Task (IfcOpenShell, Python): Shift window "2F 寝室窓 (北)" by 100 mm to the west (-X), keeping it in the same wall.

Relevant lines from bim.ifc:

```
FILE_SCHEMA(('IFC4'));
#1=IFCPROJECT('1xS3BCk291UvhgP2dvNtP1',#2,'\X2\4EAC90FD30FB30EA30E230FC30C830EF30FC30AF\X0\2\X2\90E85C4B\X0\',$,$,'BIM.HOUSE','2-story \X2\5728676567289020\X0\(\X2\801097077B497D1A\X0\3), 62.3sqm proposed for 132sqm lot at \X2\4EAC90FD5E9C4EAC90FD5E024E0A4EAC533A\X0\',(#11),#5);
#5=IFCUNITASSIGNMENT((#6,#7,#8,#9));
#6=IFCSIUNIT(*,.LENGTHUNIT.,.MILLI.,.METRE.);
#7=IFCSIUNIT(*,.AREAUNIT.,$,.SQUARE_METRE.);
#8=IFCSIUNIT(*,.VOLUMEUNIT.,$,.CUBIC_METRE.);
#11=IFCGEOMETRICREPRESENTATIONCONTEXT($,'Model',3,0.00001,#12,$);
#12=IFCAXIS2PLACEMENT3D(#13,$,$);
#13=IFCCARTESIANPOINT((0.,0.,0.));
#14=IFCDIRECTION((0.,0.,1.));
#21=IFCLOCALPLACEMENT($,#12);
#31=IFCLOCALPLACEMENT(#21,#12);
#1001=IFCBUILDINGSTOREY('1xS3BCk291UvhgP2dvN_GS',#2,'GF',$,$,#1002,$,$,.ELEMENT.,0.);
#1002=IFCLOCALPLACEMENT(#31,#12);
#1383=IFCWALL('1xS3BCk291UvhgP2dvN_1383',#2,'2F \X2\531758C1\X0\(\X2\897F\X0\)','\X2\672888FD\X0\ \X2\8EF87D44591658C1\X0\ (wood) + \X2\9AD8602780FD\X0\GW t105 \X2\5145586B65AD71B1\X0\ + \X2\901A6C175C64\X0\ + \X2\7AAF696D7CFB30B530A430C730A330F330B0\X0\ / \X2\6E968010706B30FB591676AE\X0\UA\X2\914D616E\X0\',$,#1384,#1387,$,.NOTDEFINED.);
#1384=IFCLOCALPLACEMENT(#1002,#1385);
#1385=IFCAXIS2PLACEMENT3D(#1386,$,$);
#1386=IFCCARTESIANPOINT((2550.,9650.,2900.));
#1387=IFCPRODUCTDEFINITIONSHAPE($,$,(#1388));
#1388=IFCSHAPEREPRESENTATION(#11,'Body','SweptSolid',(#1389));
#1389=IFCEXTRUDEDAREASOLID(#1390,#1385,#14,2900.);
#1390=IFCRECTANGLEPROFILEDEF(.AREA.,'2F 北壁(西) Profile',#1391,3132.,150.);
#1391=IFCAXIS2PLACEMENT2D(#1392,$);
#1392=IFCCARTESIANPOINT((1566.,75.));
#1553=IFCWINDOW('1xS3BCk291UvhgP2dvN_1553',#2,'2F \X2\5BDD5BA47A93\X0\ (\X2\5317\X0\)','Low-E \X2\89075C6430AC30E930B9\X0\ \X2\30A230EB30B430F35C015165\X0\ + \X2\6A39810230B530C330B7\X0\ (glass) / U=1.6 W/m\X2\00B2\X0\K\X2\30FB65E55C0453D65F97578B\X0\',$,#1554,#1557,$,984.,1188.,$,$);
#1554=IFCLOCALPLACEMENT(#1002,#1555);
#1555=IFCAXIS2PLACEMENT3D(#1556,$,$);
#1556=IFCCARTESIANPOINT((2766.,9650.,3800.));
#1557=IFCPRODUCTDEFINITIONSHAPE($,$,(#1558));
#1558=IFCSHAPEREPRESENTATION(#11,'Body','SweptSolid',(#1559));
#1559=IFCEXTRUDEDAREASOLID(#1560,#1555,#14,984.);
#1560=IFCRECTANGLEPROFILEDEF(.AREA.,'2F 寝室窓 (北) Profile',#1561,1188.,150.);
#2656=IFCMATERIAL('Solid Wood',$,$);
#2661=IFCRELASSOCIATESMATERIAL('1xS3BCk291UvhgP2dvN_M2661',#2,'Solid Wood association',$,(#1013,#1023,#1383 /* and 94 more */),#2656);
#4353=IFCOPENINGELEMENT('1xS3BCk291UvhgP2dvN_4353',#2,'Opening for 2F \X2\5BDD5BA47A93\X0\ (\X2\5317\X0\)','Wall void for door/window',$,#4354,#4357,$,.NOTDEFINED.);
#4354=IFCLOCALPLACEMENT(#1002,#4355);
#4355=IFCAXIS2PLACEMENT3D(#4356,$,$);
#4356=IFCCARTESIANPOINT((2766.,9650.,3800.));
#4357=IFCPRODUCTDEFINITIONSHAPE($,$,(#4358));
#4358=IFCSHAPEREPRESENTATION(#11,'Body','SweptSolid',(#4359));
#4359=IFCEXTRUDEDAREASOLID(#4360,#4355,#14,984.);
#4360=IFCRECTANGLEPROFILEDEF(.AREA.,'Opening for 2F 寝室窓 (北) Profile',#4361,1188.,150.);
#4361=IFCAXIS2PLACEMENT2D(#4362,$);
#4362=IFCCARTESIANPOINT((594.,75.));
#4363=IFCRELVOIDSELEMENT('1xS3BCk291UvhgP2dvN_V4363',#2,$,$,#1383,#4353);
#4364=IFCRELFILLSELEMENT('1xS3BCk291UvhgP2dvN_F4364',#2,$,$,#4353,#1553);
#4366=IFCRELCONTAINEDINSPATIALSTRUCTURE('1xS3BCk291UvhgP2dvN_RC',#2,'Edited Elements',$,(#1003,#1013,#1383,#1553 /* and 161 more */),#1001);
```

```python
import ifcopenshell
import ifcopenshell.api.geometry
import ifcopenshell.util.placement
import ifcopenshell.util.unit

model = ifcopenshell.open("bim.ifc")
unit_scale = ifcopenshell.util.unit.calculate_unit_scale(model)

window = model.by_guid("1xS3BCk291UvhgP2dvN_1553")
opening = window.FillsVoids[0].RelatingOpeningElement
wall = opening.VoidsElements[0].RelatingBuildingElement

wall_matrix = ifcopenshell.util.placement.get_local_placement(wall.ObjectPlacement)
shift = wall_matrix[:3, 0] * -0.1 / unit_scale
before = ifcopenshell.util.placement.get_local_placement(window.ObjectPlacement)[:3, 3].copy()

# The window is not placed relative to its opening, so move both.
for product in (opening, window):
    matrix = ifcopenshell.util.placement.get_local_placement(product.ObjectPlacement)
    matrix[:3, 3] += shift
    ifcopenshell.api.geometry.edit_object_placement(model, product=product, matrix=matrix, is_si=False)

after = ifcopenshell.util.placement.get_local_placement(window.ObjectPlacement)[:3, 3]
print("window moved by", (after - before).round(3) + 0.0)

model.write("bim_updated.ifc")
```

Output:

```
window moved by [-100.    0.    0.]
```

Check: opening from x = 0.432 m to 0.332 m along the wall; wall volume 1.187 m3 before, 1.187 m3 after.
